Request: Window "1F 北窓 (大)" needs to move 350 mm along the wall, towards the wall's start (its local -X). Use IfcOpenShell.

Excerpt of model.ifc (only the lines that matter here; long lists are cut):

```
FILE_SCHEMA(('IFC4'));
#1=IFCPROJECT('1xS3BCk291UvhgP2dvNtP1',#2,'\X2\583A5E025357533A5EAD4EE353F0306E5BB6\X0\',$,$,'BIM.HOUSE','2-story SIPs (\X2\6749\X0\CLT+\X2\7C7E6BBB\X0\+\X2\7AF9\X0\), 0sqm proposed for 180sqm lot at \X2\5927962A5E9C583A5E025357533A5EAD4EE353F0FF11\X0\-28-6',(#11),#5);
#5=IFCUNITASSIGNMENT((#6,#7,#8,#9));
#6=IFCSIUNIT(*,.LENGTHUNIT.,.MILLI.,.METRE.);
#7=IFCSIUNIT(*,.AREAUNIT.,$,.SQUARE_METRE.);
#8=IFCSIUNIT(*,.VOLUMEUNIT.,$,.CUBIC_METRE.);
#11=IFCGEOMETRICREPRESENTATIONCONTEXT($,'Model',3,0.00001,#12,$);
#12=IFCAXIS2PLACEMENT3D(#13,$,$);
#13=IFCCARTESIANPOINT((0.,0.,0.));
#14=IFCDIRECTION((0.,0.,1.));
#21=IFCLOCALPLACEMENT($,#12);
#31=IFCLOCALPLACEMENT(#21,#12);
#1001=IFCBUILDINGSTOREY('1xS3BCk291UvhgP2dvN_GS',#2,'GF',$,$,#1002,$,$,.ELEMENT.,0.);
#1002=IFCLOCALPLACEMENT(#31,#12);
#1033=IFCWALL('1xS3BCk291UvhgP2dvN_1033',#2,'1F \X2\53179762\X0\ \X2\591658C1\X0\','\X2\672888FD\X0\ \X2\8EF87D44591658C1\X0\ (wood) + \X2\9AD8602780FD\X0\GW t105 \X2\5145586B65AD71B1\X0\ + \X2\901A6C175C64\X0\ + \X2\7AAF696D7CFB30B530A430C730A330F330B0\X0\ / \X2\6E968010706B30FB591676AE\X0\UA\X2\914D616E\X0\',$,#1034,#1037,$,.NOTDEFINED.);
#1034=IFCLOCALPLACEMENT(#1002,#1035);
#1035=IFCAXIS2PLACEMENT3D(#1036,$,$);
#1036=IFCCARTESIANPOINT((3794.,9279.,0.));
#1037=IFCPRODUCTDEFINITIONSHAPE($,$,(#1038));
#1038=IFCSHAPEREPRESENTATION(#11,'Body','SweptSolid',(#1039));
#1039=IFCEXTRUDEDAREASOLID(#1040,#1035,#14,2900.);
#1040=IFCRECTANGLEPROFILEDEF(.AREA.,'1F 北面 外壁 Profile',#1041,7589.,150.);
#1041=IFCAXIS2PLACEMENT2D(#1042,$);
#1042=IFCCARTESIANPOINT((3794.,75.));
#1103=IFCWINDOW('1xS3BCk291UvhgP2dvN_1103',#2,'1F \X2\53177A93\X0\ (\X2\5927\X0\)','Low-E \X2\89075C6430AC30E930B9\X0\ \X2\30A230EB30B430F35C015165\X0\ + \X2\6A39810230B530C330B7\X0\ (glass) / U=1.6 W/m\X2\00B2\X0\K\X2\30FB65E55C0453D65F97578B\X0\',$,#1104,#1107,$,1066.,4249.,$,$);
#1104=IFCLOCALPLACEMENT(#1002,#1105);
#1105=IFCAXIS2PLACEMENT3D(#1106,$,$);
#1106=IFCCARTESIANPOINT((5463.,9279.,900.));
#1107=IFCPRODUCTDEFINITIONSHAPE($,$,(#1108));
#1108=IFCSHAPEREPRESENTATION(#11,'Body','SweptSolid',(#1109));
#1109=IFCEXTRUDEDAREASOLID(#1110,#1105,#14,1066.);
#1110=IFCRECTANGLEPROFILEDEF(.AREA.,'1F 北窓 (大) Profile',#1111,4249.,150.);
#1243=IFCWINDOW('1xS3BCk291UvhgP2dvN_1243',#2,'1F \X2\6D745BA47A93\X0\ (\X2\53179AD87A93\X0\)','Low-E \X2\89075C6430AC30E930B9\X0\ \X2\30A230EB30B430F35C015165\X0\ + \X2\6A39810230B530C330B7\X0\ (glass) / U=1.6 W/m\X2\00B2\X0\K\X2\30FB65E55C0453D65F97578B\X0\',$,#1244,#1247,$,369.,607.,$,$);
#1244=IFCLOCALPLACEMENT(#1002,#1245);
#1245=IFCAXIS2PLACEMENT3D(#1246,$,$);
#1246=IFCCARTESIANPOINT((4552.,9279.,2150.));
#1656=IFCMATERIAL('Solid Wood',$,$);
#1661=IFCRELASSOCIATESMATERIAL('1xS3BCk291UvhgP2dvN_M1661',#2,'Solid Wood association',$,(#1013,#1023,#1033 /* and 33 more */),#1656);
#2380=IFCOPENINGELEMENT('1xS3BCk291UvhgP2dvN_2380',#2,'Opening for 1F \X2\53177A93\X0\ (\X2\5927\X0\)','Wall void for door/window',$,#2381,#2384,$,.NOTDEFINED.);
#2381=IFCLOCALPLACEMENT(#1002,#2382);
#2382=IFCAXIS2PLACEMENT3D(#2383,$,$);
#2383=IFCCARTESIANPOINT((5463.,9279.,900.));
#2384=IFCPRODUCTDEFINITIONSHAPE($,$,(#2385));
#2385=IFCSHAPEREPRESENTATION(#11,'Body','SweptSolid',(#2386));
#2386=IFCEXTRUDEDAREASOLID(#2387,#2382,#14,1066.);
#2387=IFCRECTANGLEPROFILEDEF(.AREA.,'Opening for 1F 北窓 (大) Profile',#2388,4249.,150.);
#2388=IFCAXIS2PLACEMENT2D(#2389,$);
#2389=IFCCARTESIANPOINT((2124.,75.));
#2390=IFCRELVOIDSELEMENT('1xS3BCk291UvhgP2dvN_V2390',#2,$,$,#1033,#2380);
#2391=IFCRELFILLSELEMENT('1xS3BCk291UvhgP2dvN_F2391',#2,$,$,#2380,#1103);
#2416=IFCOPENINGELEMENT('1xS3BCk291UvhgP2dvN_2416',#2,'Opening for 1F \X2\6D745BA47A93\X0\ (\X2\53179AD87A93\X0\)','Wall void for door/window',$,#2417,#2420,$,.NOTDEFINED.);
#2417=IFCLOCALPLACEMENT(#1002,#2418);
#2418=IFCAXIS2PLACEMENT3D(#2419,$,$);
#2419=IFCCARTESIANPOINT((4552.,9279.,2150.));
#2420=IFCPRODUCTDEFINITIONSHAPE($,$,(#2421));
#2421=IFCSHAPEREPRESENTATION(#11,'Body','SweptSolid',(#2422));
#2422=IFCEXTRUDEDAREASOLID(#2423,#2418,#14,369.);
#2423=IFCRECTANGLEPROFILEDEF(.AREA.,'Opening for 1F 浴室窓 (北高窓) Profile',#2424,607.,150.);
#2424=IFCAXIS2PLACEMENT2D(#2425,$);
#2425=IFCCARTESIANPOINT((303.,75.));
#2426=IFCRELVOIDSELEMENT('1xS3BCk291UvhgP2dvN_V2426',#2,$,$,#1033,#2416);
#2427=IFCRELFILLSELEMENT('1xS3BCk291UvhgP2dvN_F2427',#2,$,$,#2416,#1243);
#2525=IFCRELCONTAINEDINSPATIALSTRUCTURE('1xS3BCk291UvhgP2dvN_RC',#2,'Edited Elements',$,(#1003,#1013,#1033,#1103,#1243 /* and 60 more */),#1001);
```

```python
import ifcopenshell
import ifcopenshell.api.geometry
import ifcopenshell.util.placement

model = ifcopenshell.open("model.ifc")

window = model.by_guid("1xS3BCk291UvhgP2dvN_1103")
opening = window.FillsVoids[0].RelatingOpeningElement
wall = opening.VoidsElements[0].RelatingBuildingElement

wall_matrix = ifcopenshell.util.placement.get_local_placement(wall.ObjectPlacement)
shift = wall_matrix[:3, 0] * -350.0
before = ifcopenshell.util.placement.get_local_placement(window.ObjectPlacement)[:3, 3].copy()

# The window is not placed relative to its opening, so move both.
for product in (opening, window):
    matrix = ifcopenshell.util.placement.get_local_placement(product.ObjectPlacement)
    matrix[:3, 3] += shift
    ifcopenshell.api.geometry.edit_object_placement(model, product=product, matrix=matrix, is_si=False)

after = ifcopenshell.util.placement.get_local_placement(window.ObjectPlacement)[:3, 3]
print("window moved by", (after - before).round(3) + 0.0)

model.write("model_updated.ifc")
```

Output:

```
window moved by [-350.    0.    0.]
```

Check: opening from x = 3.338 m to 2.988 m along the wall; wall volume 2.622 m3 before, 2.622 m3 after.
